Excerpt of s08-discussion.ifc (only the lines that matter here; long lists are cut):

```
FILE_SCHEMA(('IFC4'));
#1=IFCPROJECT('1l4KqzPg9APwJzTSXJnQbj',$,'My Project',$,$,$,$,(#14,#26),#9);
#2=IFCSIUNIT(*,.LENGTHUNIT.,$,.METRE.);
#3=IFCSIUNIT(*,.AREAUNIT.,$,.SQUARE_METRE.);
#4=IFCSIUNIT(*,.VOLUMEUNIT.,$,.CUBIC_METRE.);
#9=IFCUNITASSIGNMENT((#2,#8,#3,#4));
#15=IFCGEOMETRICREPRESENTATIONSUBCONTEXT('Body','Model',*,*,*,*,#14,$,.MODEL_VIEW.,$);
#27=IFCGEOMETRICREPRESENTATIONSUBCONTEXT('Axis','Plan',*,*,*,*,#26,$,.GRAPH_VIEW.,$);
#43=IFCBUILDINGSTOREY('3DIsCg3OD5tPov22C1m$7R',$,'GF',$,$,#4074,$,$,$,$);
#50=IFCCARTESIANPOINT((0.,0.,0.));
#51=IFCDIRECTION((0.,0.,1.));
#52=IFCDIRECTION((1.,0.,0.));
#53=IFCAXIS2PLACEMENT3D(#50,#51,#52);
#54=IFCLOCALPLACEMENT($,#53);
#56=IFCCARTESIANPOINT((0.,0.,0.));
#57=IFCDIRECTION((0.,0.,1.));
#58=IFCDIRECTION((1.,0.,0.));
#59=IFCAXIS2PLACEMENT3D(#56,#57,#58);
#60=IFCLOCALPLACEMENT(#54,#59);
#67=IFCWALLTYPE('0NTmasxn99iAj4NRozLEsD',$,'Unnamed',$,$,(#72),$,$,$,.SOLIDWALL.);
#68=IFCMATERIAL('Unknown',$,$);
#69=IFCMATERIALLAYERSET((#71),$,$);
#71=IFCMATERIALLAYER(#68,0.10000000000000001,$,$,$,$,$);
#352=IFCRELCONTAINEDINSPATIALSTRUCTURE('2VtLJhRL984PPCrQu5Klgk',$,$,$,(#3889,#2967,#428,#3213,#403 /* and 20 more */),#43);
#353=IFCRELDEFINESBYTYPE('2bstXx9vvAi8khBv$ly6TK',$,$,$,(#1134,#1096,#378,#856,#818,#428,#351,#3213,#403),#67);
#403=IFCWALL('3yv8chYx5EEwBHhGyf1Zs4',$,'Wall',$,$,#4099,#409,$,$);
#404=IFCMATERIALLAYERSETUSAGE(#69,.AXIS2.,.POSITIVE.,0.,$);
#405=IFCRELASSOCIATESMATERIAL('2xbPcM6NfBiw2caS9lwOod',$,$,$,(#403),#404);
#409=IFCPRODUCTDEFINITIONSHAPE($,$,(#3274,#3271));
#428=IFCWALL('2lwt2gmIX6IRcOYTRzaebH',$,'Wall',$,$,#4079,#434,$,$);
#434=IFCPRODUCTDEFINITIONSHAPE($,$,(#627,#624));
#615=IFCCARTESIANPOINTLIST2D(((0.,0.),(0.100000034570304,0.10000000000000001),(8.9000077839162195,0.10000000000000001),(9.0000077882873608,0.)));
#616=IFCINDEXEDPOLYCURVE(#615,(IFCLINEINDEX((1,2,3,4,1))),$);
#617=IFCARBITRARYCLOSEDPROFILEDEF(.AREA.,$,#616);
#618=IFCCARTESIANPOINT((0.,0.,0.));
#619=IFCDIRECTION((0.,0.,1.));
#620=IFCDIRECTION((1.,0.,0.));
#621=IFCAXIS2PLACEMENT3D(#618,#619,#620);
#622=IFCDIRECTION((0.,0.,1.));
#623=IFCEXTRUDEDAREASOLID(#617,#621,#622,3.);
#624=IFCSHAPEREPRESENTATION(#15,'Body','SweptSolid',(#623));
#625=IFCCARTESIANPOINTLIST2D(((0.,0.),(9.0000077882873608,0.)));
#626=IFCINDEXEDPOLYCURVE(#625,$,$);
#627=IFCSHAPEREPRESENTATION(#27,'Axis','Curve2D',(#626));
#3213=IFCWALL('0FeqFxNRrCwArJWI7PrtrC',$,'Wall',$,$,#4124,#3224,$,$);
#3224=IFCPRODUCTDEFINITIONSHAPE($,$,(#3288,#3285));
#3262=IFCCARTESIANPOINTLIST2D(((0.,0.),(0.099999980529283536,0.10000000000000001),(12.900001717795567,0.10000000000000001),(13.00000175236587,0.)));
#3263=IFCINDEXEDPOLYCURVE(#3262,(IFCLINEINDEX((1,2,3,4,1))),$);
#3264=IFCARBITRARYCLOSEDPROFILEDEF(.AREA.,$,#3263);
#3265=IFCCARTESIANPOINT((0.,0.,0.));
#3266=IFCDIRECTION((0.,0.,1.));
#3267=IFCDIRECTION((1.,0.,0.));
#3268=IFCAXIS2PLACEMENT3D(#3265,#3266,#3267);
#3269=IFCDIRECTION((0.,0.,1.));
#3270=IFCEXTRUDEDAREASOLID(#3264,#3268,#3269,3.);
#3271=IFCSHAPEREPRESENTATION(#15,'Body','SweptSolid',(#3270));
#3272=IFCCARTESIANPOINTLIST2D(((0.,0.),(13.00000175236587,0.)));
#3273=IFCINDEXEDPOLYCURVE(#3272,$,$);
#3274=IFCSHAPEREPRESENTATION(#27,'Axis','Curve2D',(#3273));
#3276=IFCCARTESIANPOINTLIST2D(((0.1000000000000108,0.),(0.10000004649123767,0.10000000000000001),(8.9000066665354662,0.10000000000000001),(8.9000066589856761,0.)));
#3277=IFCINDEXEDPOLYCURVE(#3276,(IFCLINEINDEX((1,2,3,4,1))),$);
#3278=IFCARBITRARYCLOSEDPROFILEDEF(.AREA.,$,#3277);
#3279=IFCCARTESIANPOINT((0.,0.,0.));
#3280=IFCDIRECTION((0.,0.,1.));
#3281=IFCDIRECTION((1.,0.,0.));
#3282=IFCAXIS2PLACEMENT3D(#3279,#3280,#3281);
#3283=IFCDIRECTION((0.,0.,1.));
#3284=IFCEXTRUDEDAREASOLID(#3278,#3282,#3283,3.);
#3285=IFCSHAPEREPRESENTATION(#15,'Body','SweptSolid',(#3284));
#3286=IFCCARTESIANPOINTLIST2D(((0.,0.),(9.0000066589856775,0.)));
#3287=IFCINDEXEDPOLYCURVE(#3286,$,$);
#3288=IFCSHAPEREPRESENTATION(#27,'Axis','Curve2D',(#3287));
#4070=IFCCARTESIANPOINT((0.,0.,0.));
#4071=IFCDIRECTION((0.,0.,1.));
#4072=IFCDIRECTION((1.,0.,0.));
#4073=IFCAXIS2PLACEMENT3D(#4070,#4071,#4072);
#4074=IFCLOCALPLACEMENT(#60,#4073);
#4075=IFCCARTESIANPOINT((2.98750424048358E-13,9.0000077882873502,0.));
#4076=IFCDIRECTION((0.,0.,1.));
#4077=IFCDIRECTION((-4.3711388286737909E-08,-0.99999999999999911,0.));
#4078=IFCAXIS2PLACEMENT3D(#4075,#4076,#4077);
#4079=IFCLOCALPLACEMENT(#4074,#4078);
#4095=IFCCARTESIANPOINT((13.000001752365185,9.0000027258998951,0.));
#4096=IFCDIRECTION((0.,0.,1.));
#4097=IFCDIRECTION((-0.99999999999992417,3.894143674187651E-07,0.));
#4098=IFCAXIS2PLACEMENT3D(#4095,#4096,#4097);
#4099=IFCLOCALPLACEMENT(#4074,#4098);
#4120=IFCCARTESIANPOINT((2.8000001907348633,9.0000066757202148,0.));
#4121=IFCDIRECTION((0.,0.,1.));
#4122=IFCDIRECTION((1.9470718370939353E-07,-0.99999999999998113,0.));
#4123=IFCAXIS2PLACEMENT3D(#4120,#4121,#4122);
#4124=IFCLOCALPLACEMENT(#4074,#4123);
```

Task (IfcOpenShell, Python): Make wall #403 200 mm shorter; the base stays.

```python
import ifcopenshell
import ifcopenshell.geom
import ifcopenshell.util.representation
import ifcopenshell.util.shape
import ifcopenshell.util.unit

model = ifcopenshell.open("s08-discussion.ifc")
unit_scale = ifcopenshell.util.unit.calculate_unit_scale(model)
settings = ifcopenshell.geom.settings()


def volume(element):
    """Net volume in cubic metres, openings subtracted."""
    shape = ifcopenshell.geom.create_shape(settings, element)
    return ifcopenshell.util.shape.get_volume(shape.geometry)


wall = model.by_guid("3yv8chYx5EEwBHhGyf1Zs4")
before = volume(wall)

body = ifcopenshell.util.representation.get_representation(wall, "Model", "Body")
solid = body.Items[0]
old_height = solid.Depth
solid.Depth -= 0.2 / unit_scale
after = volume(wall)

print(f"height {old_height:g} -> {solid.Depth:g}, volume {before:.3f} -> {after:.3f} m3")

model.write("s08-discussion_v2.ifc")
```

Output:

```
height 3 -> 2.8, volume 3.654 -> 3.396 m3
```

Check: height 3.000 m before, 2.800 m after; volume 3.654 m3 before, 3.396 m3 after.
